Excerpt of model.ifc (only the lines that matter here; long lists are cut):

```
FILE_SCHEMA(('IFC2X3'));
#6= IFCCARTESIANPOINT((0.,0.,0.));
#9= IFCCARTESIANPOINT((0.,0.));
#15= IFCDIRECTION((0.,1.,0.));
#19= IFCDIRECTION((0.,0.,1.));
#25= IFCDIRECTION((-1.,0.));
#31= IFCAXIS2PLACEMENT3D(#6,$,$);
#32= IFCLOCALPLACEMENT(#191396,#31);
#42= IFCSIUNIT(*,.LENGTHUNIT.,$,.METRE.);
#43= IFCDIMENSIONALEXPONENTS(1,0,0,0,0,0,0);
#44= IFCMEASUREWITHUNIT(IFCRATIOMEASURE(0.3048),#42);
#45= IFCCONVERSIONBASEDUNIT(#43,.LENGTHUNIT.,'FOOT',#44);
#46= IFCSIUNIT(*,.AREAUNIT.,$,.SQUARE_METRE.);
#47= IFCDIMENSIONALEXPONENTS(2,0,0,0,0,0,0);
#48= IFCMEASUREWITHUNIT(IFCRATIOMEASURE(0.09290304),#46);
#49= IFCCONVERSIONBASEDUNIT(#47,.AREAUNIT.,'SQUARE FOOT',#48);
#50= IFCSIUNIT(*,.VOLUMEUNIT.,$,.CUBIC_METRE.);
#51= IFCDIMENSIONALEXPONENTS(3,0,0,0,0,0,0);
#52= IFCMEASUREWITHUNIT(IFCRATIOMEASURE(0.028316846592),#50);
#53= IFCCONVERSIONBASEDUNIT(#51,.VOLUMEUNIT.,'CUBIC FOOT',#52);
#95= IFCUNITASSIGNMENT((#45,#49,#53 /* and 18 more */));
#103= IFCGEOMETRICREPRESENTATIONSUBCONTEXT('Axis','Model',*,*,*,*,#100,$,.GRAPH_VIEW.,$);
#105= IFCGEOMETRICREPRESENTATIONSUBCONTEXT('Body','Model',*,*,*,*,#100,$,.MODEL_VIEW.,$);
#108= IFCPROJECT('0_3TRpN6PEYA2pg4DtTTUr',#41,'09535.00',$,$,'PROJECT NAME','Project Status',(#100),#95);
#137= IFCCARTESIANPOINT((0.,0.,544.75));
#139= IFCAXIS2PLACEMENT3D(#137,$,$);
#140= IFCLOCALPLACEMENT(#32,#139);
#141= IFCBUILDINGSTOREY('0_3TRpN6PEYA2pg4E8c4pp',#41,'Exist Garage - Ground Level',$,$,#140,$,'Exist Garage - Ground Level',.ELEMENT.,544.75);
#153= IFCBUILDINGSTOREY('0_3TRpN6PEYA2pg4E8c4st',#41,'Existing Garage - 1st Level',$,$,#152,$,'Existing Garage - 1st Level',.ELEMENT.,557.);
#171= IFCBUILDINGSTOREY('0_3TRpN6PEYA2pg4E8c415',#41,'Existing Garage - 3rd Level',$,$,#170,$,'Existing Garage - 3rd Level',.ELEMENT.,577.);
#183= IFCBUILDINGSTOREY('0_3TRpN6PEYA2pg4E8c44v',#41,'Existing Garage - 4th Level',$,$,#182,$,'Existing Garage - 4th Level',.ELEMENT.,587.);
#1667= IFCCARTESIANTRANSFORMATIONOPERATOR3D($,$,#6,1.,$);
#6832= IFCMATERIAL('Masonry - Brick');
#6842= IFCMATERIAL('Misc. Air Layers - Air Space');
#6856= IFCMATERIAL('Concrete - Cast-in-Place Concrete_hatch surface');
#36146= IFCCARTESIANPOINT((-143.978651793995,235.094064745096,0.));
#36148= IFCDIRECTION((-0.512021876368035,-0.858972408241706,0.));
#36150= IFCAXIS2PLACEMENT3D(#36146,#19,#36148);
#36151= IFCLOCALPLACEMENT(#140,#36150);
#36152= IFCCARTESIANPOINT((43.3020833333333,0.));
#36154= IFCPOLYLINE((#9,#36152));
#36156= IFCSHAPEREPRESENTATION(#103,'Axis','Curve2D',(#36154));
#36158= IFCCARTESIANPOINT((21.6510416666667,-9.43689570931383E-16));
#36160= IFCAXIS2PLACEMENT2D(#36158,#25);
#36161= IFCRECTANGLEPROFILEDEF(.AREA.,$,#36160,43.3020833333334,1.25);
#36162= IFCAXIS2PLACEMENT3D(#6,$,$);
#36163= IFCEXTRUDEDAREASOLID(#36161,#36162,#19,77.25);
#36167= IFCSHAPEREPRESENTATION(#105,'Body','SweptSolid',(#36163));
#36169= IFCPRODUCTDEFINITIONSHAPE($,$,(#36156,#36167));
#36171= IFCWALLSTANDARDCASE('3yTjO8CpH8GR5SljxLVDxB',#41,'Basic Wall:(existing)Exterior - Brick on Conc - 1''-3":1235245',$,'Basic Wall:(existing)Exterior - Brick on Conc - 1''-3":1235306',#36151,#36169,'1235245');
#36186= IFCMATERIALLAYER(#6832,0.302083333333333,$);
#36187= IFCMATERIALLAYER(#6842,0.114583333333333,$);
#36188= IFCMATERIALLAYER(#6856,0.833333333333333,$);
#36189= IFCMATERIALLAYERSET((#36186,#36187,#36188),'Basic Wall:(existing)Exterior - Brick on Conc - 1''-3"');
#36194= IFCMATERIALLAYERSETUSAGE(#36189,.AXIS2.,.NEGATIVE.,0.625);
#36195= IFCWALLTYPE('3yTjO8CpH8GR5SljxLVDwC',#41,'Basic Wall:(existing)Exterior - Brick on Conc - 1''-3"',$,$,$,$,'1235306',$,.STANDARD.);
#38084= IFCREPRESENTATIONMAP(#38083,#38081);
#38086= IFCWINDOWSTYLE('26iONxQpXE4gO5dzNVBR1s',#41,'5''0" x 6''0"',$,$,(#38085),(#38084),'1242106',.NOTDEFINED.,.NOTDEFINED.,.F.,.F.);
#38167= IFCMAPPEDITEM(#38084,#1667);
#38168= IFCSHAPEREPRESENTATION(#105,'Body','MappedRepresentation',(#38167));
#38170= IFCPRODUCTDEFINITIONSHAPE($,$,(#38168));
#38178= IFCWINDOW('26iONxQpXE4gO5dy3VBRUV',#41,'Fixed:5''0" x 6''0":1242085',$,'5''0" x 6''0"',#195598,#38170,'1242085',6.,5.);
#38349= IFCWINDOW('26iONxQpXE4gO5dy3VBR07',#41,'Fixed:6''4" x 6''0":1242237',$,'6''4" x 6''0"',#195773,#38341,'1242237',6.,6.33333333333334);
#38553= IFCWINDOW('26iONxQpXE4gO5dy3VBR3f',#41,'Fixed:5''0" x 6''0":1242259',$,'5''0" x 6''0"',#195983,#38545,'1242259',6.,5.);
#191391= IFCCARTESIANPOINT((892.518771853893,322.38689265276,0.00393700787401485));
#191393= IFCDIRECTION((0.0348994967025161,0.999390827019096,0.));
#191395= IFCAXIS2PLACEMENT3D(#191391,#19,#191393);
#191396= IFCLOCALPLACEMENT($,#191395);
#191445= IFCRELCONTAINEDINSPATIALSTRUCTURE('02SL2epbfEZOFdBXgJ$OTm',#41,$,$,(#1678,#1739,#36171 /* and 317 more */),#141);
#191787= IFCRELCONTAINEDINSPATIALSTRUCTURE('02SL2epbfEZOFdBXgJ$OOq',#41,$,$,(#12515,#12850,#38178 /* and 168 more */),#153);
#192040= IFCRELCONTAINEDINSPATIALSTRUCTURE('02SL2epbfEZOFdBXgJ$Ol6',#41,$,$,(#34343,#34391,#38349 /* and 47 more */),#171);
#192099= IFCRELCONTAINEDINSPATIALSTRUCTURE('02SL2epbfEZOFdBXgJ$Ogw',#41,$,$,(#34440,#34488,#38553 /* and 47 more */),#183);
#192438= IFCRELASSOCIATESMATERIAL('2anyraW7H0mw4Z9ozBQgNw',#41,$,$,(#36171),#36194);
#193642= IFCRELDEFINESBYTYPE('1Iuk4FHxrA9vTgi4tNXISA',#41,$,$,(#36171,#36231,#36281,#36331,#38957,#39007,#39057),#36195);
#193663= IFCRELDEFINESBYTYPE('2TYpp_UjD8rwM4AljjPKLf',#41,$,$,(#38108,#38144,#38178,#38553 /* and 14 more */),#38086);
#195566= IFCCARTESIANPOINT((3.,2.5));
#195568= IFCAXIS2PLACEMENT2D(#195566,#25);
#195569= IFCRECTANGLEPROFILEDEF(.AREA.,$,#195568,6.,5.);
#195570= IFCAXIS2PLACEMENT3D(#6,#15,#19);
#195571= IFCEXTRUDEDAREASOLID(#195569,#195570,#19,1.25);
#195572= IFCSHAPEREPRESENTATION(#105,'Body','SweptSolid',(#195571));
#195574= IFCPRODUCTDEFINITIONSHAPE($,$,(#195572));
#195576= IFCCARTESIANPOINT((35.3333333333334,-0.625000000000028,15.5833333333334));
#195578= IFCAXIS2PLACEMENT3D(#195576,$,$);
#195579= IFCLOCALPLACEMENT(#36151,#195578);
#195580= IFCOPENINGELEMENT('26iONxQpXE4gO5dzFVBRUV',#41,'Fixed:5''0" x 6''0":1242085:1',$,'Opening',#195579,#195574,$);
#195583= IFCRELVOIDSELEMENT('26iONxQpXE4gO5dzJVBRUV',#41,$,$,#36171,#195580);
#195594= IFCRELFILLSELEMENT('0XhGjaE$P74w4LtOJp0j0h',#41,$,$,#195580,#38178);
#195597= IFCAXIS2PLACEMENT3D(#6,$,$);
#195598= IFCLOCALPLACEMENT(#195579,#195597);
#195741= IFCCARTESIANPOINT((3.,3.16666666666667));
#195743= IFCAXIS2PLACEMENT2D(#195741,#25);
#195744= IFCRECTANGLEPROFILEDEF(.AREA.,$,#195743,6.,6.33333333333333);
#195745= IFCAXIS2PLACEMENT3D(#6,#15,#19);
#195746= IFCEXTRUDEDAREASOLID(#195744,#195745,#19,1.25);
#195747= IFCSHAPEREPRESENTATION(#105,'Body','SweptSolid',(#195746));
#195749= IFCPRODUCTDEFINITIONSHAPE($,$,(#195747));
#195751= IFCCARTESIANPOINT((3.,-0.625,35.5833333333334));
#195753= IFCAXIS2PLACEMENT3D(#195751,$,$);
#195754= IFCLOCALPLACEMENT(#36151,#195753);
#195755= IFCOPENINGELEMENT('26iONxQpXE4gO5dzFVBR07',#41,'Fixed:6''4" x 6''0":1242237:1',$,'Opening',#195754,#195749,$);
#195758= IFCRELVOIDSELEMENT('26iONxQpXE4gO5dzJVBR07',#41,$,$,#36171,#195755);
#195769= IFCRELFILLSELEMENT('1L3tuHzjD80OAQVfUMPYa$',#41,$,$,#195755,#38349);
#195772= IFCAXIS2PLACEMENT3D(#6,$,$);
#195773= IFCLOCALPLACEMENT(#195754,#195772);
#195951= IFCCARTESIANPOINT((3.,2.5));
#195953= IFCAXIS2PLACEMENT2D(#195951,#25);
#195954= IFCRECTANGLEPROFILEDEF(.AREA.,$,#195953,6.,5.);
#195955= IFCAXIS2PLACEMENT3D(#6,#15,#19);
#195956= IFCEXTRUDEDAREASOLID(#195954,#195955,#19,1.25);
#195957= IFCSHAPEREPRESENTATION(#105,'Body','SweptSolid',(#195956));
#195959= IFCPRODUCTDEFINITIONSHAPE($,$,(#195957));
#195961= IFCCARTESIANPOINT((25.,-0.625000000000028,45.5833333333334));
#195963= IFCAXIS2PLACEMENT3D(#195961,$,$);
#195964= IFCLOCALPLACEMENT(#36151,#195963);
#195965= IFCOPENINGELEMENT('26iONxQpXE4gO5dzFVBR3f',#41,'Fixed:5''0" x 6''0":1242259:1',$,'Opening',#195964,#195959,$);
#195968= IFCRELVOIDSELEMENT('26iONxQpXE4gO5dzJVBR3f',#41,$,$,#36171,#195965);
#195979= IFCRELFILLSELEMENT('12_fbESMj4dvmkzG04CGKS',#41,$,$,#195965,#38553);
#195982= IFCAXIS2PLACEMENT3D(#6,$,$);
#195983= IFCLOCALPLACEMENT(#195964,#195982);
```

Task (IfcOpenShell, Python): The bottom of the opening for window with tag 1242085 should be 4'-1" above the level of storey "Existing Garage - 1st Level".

```python
import numpy as np
import ifcopenshell
import ifcopenshell.api.geometry
import ifcopenshell.geom
import ifcopenshell.util.element
import ifcopenshell.util.placement
import ifcopenshell.util.shape
import ifcopenshell.util.unit

model = ifcopenshell.open("model.ifc")
unit_scale = ifcopenshell.util.unit.calculate_unit_scale(model)

window = model.by_id(38178)
opening = window.FillsVoids[0].RelatingOpeningElement
storey = ifcopenshell.util.element.get_container(window, ifc_class="IfcBuildingStorey")
level = ifcopenshell.util.placement.get_local_placement(storey.ObjectPlacement)[2, 3]

# The opening's origin need not be at the sill, so measure its lowest point.
shape = ifcopenshell.geom.create_shape(ifcopenshell.geom.settings(), opening)
bottom = ifcopenshell.util.shape.get_shape_bottom_elevation(shape, shape.geometry) / unit_scale
dz = level + 49 * 0.0254 / unit_scale - bottom

shift = np.array([0.0, 0.0, dz])
# The window is placed relative to its opening, so it follows when the opening moves.
matrix = ifcopenshell.util.placement.get_local_placement(opening.ObjectPlacement)
matrix[:3, 3] += shift
ifcopenshell.api.geometry.edit_object_placement(
    model, product=opening, matrix=matrix, is_si=False, should_transform_children=True
)

print(f"moved by {dz * unit_scale:+.3f} m")

model.write("model-out.ifc")
```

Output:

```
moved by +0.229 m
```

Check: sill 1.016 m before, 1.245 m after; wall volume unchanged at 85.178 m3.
